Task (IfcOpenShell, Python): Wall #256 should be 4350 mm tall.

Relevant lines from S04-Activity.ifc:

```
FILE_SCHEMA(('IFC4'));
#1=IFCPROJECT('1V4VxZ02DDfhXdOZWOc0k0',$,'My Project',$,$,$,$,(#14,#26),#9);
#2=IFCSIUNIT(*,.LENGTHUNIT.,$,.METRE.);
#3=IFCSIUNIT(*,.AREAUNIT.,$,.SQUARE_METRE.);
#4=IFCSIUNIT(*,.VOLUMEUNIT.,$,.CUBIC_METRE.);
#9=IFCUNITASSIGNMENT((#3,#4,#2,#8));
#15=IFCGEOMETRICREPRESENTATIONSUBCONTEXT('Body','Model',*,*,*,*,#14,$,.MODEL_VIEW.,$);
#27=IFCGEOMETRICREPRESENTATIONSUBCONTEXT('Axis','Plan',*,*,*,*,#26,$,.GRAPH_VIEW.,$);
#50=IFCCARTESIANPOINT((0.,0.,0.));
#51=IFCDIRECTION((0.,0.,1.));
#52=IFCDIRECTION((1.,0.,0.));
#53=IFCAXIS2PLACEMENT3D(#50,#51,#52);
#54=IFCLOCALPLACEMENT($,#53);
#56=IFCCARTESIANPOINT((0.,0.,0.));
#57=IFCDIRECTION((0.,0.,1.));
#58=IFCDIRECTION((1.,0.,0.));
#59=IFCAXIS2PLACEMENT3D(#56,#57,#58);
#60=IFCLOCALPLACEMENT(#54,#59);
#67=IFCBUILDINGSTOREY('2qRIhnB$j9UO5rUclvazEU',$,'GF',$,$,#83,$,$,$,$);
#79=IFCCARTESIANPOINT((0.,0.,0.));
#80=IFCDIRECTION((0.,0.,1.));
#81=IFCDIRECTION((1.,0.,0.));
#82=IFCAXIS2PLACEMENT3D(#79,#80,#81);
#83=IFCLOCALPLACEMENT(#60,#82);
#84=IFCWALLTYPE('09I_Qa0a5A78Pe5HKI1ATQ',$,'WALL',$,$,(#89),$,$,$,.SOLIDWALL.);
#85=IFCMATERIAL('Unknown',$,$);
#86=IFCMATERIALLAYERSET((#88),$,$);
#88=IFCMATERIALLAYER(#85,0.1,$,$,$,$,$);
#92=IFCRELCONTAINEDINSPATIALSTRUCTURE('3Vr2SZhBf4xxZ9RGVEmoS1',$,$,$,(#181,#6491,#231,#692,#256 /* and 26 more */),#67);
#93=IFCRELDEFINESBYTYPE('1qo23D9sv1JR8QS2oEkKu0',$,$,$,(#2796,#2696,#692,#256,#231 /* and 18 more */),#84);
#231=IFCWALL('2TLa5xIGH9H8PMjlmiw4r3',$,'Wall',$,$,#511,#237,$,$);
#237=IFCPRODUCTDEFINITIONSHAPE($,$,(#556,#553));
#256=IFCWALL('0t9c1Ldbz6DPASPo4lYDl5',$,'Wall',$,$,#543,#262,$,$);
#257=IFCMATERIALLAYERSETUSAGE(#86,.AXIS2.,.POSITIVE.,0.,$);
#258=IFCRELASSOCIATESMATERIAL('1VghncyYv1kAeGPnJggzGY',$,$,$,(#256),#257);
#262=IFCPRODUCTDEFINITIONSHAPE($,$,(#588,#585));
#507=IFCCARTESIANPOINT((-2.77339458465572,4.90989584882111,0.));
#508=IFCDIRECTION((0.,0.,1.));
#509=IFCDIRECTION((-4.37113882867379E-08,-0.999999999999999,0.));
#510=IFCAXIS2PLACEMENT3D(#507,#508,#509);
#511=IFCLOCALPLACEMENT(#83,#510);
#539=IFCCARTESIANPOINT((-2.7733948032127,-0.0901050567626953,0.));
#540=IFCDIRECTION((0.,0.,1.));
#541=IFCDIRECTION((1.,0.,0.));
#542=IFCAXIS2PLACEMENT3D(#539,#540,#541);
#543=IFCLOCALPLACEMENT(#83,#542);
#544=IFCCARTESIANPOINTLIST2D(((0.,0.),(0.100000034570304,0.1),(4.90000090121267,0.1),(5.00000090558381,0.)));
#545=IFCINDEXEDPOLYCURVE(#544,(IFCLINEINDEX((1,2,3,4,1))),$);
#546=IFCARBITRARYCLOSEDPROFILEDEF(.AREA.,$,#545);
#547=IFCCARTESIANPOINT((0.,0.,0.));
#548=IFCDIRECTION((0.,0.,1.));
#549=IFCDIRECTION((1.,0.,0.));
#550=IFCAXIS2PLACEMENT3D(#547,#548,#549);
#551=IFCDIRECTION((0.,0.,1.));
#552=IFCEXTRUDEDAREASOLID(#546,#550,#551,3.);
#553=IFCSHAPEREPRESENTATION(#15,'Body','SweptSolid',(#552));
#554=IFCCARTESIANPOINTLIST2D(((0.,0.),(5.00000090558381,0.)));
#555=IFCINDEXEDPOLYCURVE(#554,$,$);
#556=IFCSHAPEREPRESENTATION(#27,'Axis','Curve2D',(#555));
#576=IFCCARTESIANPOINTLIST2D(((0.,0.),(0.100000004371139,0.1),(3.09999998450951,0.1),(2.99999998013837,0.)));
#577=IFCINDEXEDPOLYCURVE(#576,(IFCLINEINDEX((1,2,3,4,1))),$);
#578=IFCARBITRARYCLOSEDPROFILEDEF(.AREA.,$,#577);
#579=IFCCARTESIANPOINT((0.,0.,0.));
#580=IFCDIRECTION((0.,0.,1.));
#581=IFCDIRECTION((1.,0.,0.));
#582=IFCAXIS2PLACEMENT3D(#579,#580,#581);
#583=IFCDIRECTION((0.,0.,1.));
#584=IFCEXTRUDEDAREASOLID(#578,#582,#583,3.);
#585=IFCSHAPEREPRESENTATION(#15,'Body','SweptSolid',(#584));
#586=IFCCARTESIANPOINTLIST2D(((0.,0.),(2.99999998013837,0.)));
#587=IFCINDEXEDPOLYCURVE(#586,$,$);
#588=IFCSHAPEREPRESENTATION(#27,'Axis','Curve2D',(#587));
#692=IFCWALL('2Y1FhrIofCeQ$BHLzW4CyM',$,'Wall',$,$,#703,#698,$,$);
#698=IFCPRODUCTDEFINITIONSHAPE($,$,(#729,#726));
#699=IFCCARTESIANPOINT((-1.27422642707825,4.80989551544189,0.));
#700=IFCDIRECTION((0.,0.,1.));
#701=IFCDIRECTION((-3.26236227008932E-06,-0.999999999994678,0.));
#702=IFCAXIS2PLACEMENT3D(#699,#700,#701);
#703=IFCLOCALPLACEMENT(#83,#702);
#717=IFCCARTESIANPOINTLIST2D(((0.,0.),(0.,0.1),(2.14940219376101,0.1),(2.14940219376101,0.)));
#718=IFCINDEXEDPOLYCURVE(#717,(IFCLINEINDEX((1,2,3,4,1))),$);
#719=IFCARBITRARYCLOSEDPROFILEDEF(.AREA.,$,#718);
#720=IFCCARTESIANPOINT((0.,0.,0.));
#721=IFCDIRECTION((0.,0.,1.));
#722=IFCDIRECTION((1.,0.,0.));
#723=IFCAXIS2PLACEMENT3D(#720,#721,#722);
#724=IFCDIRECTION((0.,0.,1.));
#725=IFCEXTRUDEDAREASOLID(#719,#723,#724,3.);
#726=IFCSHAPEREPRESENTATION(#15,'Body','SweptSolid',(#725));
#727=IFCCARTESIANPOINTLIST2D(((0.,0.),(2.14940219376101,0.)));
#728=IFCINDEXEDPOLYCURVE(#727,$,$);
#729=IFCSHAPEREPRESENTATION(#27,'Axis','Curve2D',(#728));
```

```python
import ifcopenshell
import ifcopenshell.geom
import ifcopenshell.util.representation
import ifcopenshell.util.shape

model = ifcopenshell.open("S04-Activity.ifc")
settings = ifcopenshell.geom.settings()


def volume(element):
    """Net volume in cubic metres, openings subtracted."""
    shape = ifcopenshell.geom.create_shape(settings, element)
    return ifcopenshell.util.shape.get_volume(shape.geometry)


wall = model.by_guid("0t9c1Ldbz6DPASPo4lYDl5")
before = volume(wall)

body = ifcopenshell.util.representation.get_representation(wall, "Model", "Body")
solid = body.Items[0]
old_height = solid.Depth
solid.Depth = 4.35
after = volume(wall)

print(f"height {old_height:g} -> {solid.Depth:g}, volume {before:.3f} -> {after:.3f} m3")

model.write("S04-Activity_rev.ifc")
```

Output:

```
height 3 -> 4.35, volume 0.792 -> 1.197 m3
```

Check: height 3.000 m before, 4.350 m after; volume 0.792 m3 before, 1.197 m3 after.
